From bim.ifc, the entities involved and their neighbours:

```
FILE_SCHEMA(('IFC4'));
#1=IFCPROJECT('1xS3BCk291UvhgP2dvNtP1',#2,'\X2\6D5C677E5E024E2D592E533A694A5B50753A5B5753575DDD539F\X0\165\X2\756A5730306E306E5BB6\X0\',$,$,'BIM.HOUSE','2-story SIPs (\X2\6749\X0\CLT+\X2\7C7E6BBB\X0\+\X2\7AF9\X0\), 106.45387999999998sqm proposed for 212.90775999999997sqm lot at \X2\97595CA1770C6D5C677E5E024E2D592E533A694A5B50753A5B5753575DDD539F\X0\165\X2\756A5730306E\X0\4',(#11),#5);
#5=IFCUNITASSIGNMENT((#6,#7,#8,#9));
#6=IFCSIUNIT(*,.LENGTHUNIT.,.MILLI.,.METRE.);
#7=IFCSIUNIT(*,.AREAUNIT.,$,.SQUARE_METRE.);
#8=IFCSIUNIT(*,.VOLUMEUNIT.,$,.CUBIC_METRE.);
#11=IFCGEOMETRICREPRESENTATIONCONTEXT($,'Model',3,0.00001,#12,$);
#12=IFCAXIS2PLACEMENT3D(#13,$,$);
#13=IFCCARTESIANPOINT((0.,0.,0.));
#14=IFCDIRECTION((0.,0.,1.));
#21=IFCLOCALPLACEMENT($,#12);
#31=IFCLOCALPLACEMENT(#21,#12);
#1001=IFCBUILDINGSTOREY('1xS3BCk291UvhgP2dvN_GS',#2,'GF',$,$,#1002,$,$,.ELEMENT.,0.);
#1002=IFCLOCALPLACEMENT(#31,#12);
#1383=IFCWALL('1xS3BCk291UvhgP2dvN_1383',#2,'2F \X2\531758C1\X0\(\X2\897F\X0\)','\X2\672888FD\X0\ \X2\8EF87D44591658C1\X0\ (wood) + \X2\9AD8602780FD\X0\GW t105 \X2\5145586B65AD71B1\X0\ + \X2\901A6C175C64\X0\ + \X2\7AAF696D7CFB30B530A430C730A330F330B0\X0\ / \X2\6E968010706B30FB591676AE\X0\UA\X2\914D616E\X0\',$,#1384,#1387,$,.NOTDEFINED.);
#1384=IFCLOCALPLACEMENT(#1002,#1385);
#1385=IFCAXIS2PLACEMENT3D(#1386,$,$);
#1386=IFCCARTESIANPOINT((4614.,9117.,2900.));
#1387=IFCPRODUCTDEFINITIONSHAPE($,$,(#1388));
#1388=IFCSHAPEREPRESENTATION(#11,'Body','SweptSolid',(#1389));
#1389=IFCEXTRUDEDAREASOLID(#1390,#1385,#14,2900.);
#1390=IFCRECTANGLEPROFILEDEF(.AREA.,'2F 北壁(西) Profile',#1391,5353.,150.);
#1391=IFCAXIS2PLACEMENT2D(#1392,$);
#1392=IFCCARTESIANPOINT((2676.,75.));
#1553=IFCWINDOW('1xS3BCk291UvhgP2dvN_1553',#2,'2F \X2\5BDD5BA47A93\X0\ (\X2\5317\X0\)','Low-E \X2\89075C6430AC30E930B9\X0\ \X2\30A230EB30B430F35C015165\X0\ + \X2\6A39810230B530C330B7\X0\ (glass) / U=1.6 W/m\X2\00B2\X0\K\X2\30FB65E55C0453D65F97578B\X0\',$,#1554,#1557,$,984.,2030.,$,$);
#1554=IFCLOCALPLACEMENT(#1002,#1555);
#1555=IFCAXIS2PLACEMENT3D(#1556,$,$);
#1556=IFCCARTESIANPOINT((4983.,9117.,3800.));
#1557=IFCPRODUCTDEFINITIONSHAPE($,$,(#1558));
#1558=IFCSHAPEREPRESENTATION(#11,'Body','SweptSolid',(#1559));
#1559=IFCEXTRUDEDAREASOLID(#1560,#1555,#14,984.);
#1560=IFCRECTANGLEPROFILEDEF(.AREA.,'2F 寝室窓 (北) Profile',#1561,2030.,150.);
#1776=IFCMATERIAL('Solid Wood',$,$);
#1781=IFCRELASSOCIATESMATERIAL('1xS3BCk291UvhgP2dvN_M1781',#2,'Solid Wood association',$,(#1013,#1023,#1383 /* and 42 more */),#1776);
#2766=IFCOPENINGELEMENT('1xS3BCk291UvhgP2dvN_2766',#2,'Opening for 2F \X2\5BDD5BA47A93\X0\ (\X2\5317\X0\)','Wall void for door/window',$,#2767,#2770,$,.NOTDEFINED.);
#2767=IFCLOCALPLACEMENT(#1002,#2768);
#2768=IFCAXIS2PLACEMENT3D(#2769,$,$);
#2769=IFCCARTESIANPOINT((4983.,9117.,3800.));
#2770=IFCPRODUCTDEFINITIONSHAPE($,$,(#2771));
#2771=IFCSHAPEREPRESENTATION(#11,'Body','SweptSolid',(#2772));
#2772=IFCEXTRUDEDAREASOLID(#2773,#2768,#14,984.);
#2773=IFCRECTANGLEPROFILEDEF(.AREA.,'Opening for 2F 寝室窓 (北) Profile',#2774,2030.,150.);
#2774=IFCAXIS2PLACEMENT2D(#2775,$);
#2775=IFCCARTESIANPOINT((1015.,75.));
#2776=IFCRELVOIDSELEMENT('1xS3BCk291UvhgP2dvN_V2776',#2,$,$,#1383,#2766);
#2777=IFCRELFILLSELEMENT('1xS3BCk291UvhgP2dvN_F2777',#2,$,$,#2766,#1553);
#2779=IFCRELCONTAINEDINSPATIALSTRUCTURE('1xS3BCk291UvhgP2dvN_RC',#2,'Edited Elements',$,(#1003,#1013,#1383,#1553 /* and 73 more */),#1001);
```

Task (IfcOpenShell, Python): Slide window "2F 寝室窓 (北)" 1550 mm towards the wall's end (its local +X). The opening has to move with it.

```python
import ifcopenshell
import ifcopenshell.api.geometry
import ifcopenshell.util.placement

model = ifcopenshell.open("bim.ifc")

window = model.by_guid("1xS3BCk291UvhgP2dvN_1553")
opening = window.FillsVoids[0].RelatingOpeningElement
wall = opening.VoidsElements[0].RelatingBuildingElement

wall_matrix = ifcopenshell.util.placement.get_local_placement(wall.ObjectPlacement)
shift = wall_matrix[:3, 0] * 1550.0
before = ifcopenshell.util.placement.get_local_placement(window.ObjectPlacement)[:3, 3].copy()

# The window is not placed relative to its opening, so move both.
for product in (opening, window):
    matrix = ifcopenshell.util.placement.get_local_placement(product.ObjectPlacement)
    matrix[:3, 3] += shift
    ifcopenshell.api.geometry.edit_object_placement(model, product=product, matrix=matrix, is_si=False)

after = ifcopenshell.util.placement.get_local_placement(window.ObjectPlacement)[:3, 3]
print("window moved by", (after - before).round(3) + 0.0)

model.write("bim-out.ifc")
```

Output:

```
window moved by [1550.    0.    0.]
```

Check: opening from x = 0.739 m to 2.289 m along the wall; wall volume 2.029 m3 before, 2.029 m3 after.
